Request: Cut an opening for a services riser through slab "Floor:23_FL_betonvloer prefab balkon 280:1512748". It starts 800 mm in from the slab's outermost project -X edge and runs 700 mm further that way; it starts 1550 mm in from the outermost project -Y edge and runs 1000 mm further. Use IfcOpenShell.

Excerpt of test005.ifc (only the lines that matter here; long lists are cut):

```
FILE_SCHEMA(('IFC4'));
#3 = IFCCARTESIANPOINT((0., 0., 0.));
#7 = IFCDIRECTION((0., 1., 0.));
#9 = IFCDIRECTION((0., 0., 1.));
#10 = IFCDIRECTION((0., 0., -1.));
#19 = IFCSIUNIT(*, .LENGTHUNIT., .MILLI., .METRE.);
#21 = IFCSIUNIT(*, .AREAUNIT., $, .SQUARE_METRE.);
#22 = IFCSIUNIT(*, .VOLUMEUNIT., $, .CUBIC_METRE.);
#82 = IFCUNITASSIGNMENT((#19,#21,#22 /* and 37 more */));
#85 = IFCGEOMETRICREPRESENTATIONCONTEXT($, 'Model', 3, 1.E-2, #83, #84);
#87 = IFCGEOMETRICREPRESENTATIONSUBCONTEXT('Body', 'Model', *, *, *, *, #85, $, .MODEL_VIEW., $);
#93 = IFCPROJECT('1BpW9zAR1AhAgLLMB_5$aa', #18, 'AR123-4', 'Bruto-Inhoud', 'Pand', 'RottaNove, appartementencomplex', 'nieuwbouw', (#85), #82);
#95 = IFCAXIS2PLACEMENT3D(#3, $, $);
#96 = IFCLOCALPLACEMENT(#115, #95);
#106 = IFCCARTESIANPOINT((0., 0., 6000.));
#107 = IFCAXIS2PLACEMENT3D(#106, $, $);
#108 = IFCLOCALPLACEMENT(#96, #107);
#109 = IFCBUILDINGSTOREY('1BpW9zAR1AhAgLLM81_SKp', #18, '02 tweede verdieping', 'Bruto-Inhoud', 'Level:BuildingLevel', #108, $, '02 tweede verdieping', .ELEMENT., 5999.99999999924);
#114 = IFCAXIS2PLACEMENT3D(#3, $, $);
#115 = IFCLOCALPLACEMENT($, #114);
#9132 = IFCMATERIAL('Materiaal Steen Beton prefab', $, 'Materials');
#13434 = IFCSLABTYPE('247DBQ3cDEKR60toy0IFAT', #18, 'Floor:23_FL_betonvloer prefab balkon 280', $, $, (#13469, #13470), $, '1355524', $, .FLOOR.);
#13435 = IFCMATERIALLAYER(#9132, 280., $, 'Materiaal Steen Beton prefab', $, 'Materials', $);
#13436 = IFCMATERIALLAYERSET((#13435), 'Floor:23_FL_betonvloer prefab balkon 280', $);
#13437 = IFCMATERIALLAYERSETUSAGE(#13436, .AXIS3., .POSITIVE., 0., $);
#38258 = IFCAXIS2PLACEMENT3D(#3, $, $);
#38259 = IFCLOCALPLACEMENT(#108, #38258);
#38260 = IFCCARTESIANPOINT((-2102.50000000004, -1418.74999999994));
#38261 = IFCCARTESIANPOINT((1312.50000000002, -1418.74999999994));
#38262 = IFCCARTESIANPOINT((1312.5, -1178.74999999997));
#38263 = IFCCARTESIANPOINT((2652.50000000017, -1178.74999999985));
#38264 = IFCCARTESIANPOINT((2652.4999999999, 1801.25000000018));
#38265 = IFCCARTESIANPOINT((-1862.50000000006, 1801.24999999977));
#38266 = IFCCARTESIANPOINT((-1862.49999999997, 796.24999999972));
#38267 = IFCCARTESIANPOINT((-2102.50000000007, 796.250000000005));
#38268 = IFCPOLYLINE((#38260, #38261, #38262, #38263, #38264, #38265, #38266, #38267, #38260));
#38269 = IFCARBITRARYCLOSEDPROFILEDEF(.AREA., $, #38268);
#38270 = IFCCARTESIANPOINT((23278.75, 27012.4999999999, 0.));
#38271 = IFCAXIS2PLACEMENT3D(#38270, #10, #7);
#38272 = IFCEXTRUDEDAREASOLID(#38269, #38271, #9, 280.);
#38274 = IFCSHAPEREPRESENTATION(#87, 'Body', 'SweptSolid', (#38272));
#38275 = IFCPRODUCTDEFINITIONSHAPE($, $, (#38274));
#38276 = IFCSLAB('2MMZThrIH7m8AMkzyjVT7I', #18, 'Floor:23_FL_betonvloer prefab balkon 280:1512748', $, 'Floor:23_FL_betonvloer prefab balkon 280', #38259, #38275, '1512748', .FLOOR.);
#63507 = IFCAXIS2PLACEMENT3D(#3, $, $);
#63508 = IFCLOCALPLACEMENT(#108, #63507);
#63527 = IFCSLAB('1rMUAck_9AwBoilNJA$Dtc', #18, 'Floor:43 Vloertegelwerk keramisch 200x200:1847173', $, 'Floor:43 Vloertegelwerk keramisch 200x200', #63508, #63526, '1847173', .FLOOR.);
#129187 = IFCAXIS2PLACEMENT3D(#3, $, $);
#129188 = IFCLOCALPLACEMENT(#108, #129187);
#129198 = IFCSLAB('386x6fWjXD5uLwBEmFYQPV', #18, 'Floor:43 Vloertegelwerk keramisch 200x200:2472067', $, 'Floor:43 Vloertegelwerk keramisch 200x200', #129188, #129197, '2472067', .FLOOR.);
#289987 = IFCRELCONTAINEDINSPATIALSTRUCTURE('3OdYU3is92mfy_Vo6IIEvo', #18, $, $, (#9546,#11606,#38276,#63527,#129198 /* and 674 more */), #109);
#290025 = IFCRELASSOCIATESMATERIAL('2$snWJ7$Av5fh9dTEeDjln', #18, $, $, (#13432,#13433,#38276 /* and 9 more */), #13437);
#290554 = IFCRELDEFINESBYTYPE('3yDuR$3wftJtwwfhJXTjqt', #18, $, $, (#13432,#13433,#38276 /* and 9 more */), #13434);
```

```python
import numpy as np
import ifcopenshell
import ifcopenshell.api.feature
import ifcopenshell.api.geometry
import ifcopenshell.api.root
import ifcopenshell.geom
import ifcopenshell.util.placement
import ifcopenshell.util.representation
import ifcopenshell.util.shape
import ifcopenshell.util.unit

model = ifcopenshell.open("test005.ifc")
unit_scale = ifcopenshell.util.unit.calculate_unit_scale(model)
settings = ifcopenshell.geom.settings()


def volume(element):
    """Net volume in cubic metres, openings subtracted."""
    shape = ifcopenshell.geom.create_shape(settings, element)
    return ifcopenshell.util.shape.get_volume(shape.geometry)


slab = model.by_guid("2MMZThrIH7m8AMkzyjVT7I")
before = volume(slab)

# Extent in the slab's own axes, in metres. The edges named are its -X and -Y sides.
slab_shape = ifcopenshell.geom.create_shape(settings, slab)
vertices = ifcopenshell.util.shape.get_vertices(slab_shape.geometry)
x_min, y_min, bottom = vertices.min(axis=0)
top = vertices[:, 2].max()

opening = ifcopenshell.api.root.create_entity(model, ifc_class="IfcOpeningElement", name="Services riser opening", predefined_type="OPENING")
context = ifcopenshell.util.representation.get_context(model, "Model", "Body", "MODEL_VIEW")
width, depth = 0.7, 1
outline = [(0.0, 0.0), (width, 0.0), (width, depth), (0.0, depth), (0.0, 0.0)]
# Overshoot both faces by 50 mm so the cut is clean.
shape = ifcopenshell.api.geometry.add_slab_representation(
    model, context=context, depth=top - bottom + 0.1, polyline=outline
)
ifcopenshell.api.geometry.assign_representation(model, product=opening, representation=shape)

matrix = ifcopenshell.util.placement.get_local_placement(slab.ObjectPlacement)
matrix[:, 3] = matrix @ np.append(np.array([x_min + 0.8, y_min + 1.55, bottom - 0.05]) / unit_scale, 1.0)
ifcopenshell.api.geometry.edit_object_placement(model, product=opening, matrix=matrix, is_si=False)
ifcopenshell.api.feature.add_feature(model, feature=opening, element=slab)

after = volume(slab)

print(f"slab volume {before:.3f} -> {after:.3f} m3")

model.write("test005_edited.ifc")
```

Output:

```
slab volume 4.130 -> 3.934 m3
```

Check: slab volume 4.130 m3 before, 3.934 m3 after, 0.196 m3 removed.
